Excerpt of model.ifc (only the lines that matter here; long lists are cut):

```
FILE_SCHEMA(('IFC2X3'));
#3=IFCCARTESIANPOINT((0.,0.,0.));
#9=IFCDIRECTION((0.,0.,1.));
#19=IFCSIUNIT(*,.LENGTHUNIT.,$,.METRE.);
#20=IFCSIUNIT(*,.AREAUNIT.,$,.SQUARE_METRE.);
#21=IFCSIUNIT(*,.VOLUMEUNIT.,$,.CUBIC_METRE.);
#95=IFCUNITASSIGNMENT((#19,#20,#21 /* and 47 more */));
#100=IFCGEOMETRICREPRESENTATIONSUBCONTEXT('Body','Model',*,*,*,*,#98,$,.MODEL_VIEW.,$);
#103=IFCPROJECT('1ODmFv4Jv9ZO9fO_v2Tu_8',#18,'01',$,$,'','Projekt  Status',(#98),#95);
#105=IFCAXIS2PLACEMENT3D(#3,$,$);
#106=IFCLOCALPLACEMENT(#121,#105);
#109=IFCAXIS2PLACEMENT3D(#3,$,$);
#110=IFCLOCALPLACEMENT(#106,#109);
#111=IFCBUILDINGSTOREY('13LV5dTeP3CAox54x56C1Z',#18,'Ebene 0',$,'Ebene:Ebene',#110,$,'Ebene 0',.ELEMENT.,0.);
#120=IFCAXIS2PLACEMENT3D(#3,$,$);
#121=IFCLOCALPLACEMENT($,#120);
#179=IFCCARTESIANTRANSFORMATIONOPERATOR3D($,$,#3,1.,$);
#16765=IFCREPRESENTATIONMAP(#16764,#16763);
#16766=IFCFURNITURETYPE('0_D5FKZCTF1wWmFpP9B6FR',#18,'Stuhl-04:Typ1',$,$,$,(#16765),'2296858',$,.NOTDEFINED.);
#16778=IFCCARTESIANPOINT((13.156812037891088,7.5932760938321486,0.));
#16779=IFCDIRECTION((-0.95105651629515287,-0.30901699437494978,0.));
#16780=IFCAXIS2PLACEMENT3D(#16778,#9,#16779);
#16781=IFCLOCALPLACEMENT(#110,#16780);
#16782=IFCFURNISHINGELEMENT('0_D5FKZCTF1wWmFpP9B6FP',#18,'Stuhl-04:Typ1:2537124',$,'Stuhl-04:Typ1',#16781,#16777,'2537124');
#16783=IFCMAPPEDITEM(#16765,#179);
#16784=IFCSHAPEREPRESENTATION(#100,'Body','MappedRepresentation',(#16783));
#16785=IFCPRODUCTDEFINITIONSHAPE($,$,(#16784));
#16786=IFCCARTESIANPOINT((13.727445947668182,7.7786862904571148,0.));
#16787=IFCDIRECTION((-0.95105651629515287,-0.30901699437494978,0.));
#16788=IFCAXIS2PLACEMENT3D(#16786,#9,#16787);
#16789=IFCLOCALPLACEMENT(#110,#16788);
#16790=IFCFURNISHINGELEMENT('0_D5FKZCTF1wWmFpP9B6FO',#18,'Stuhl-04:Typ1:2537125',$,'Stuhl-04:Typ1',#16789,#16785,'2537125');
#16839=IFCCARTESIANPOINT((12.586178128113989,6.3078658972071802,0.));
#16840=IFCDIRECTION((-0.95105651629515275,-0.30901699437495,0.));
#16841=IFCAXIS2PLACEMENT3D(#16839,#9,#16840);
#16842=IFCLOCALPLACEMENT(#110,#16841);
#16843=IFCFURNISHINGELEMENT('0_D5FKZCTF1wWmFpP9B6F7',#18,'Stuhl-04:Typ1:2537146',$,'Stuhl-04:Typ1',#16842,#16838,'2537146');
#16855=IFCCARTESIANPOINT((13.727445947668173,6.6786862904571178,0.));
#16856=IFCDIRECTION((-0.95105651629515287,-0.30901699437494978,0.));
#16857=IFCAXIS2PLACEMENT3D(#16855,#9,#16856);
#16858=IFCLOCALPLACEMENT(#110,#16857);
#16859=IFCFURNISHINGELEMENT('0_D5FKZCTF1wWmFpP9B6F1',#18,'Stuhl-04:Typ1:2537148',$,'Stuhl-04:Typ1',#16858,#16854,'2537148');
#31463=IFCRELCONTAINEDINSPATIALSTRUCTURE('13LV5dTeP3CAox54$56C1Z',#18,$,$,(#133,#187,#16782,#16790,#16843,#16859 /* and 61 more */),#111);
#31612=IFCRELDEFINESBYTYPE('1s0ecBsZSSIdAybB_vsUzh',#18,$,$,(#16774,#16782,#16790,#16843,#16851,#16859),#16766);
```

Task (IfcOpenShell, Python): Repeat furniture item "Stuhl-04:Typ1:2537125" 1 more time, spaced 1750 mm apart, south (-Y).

```python
import numpy as np
import ifcopenshell
import ifcopenshell.api.geometry
import ifcopenshell.api.root
import ifcopenshell.util.element
import ifcopenshell.util.placement

model = ifcopenshell.open("model.ifc")

source = model.by_id(16790)
base = ifcopenshell.util.placement.get_local_placement(source.ObjectPlacement)
step = np.array([0.0, -1.0, 0.0]) * 1.75

for i in range(1, 2):
    copy = ifcopenshell.api.root.copy_class(model, product=source)
    copy.Representation = ifcopenshell.util.element.copy_deep(
        model, source.Representation, exclude=["IfcGeometricRepresentationContext", "IfcRepresentationMap"]
    )
    copy.Name = "Stuhl-04:Typ1"
    copy.Tag = None
    matrix = base.copy()
    matrix[:3, 3] += i * step
    print("added at", matrix[:3, 3].round(3) + 0.0)
    ifcopenshell.api.geometry.edit_object_placement(model, product=copy, matrix=matrix, is_si=False)

model.write("model_edited.ifc")
```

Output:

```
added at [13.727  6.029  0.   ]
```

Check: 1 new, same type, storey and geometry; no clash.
